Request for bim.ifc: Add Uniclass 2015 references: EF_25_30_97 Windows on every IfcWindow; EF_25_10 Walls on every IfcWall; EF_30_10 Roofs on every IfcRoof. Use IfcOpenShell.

First a look at what the model holds.

```python
import ifcopenshell

model = ifcopenshell.open("bim.ifc")
print(model.schema)
print("classifications:", [c.Name for c in model.by_type("IfcClassification")])
for ifc_class in ("IfcDoor", "IfcRoof", "IfcStair", "IfcWall", "IfcWindow"):
    print(ifc_class, len(model.by_type(ifc_class)))
```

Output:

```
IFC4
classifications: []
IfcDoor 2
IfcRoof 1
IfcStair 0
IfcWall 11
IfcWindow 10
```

```python
import ifcopenshell
import ifcopenshell.api.classification

model = ifcopenshell.open("bim.ifc")

system = ifcopenshell.api.classification.add_classification(model, classification="Uniclass 2015")

codes = {
    "IfcWindow": ("EF_25_30_97", "Windows"),
    "IfcWall": ("EF_25_10", "Walls"),
    "IfcRoof": ("EF_30_10", "Roofs"),
}
for ifc_class, (code, name) in codes.items():
    products = model.by_type(ifc_class)
    ifcopenshell.api.classification.add_reference(
        model, products=products, classification=system, identification=code, name=name
    )
    print(code, len(products))

model.write("bim_rev.ifc")
```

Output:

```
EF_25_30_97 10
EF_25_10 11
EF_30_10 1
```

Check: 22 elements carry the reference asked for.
